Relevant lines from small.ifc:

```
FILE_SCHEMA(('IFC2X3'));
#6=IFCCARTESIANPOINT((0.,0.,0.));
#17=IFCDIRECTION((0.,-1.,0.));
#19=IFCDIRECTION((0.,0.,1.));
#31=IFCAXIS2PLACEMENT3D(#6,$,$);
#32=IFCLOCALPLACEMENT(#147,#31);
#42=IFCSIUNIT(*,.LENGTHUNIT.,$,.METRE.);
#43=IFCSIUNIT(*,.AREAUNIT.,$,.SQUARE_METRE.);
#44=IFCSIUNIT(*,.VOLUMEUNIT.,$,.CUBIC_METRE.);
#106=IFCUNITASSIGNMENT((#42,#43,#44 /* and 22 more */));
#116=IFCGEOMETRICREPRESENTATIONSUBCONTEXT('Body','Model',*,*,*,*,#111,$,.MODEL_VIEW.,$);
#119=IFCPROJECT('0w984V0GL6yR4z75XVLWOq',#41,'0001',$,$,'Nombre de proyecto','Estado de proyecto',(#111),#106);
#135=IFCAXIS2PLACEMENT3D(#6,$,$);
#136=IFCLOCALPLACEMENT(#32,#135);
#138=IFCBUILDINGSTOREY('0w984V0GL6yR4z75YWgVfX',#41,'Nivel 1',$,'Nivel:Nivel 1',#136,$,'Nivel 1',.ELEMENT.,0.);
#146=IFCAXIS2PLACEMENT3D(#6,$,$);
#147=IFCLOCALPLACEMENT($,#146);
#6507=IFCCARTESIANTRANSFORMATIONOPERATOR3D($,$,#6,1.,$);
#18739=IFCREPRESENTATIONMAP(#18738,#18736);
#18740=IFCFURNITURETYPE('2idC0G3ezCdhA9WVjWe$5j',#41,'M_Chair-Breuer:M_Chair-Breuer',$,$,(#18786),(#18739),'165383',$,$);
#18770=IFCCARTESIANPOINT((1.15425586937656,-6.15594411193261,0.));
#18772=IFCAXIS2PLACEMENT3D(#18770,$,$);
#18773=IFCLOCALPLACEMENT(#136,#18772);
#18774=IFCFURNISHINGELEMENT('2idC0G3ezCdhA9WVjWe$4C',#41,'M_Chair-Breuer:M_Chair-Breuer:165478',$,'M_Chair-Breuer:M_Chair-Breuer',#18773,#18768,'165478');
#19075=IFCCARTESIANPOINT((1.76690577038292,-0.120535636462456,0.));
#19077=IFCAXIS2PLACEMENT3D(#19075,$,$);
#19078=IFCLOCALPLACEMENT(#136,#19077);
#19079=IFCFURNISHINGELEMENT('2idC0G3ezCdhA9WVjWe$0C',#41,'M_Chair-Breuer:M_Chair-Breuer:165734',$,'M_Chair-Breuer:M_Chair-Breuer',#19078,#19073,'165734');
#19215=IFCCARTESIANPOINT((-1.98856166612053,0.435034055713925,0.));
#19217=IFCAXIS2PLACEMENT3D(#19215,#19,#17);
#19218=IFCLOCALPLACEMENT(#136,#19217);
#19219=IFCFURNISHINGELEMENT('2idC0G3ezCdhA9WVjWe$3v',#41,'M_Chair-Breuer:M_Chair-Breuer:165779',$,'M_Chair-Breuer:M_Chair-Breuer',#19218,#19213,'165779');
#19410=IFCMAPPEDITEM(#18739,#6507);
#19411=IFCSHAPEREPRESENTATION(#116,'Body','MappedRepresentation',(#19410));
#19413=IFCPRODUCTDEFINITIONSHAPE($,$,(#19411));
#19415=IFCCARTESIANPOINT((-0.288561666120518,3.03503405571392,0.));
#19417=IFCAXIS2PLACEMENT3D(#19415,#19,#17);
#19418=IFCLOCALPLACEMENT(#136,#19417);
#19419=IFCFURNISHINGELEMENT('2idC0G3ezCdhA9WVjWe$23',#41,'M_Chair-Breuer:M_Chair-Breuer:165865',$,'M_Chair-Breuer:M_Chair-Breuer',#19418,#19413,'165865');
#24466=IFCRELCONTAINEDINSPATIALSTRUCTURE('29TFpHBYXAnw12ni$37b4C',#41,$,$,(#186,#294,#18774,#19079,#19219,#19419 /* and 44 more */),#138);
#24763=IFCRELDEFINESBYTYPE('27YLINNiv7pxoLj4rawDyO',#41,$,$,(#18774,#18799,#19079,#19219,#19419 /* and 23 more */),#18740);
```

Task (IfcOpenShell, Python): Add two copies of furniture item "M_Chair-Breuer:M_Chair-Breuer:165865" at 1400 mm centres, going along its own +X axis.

```python
import ifcopenshell
import ifcopenshell.api.geometry
import ifcopenshell.api.root
import ifcopenshell.util.element
import ifcopenshell.util.placement

model = ifcopenshell.open("small.ifc")


def reuse_history(source, copy):
    """copy_class also copies each property set's owner history, people and application; keep the originals."""
    for rel in copy.IsDefinedBy:
        if rel.is_a("IfcRelDefinesByProperties") and (history := rel.RelatingPropertyDefinition.OwnerHistory):
            rel.RelatingPropertyDefinition.OwnerHistory = source.OwnerHistory
            ifcopenshell.util.element.remove_deep2(model, history)


source = model.by_guid("2idC0G3ezCdhA9WVjWe$23")
base = ifcopenshell.util.placement.get_local_placement(source.ObjectPlacement)
step = base[:3, 0] * 1.4

for i in range(1, 3):
    copy = ifcopenshell.api.root.copy_class(model, product=source)
    copy.Representation = ifcopenshell.util.element.copy_deep(
        model, source.Representation, exclude=["IfcGeometricRepresentationContext", "IfcRepresentationMap"]
    )
    copy.Name = "M_Chair-Breuer:M_Chair-Breuer"
    copy.Tag = None
    reuse_history(source, copy)
    matrix = base.copy()
    matrix[:3, 3] += i * step
    print("added at", matrix[:3, 3].round(3) + 0.0)
    ifcopenshell.api.geometry.edit_object_placement(model, product=copy, matrix=matrix, is_si=False)

model.write("small_rev.ifc")
```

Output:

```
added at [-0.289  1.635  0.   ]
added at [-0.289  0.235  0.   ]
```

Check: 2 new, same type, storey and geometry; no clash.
